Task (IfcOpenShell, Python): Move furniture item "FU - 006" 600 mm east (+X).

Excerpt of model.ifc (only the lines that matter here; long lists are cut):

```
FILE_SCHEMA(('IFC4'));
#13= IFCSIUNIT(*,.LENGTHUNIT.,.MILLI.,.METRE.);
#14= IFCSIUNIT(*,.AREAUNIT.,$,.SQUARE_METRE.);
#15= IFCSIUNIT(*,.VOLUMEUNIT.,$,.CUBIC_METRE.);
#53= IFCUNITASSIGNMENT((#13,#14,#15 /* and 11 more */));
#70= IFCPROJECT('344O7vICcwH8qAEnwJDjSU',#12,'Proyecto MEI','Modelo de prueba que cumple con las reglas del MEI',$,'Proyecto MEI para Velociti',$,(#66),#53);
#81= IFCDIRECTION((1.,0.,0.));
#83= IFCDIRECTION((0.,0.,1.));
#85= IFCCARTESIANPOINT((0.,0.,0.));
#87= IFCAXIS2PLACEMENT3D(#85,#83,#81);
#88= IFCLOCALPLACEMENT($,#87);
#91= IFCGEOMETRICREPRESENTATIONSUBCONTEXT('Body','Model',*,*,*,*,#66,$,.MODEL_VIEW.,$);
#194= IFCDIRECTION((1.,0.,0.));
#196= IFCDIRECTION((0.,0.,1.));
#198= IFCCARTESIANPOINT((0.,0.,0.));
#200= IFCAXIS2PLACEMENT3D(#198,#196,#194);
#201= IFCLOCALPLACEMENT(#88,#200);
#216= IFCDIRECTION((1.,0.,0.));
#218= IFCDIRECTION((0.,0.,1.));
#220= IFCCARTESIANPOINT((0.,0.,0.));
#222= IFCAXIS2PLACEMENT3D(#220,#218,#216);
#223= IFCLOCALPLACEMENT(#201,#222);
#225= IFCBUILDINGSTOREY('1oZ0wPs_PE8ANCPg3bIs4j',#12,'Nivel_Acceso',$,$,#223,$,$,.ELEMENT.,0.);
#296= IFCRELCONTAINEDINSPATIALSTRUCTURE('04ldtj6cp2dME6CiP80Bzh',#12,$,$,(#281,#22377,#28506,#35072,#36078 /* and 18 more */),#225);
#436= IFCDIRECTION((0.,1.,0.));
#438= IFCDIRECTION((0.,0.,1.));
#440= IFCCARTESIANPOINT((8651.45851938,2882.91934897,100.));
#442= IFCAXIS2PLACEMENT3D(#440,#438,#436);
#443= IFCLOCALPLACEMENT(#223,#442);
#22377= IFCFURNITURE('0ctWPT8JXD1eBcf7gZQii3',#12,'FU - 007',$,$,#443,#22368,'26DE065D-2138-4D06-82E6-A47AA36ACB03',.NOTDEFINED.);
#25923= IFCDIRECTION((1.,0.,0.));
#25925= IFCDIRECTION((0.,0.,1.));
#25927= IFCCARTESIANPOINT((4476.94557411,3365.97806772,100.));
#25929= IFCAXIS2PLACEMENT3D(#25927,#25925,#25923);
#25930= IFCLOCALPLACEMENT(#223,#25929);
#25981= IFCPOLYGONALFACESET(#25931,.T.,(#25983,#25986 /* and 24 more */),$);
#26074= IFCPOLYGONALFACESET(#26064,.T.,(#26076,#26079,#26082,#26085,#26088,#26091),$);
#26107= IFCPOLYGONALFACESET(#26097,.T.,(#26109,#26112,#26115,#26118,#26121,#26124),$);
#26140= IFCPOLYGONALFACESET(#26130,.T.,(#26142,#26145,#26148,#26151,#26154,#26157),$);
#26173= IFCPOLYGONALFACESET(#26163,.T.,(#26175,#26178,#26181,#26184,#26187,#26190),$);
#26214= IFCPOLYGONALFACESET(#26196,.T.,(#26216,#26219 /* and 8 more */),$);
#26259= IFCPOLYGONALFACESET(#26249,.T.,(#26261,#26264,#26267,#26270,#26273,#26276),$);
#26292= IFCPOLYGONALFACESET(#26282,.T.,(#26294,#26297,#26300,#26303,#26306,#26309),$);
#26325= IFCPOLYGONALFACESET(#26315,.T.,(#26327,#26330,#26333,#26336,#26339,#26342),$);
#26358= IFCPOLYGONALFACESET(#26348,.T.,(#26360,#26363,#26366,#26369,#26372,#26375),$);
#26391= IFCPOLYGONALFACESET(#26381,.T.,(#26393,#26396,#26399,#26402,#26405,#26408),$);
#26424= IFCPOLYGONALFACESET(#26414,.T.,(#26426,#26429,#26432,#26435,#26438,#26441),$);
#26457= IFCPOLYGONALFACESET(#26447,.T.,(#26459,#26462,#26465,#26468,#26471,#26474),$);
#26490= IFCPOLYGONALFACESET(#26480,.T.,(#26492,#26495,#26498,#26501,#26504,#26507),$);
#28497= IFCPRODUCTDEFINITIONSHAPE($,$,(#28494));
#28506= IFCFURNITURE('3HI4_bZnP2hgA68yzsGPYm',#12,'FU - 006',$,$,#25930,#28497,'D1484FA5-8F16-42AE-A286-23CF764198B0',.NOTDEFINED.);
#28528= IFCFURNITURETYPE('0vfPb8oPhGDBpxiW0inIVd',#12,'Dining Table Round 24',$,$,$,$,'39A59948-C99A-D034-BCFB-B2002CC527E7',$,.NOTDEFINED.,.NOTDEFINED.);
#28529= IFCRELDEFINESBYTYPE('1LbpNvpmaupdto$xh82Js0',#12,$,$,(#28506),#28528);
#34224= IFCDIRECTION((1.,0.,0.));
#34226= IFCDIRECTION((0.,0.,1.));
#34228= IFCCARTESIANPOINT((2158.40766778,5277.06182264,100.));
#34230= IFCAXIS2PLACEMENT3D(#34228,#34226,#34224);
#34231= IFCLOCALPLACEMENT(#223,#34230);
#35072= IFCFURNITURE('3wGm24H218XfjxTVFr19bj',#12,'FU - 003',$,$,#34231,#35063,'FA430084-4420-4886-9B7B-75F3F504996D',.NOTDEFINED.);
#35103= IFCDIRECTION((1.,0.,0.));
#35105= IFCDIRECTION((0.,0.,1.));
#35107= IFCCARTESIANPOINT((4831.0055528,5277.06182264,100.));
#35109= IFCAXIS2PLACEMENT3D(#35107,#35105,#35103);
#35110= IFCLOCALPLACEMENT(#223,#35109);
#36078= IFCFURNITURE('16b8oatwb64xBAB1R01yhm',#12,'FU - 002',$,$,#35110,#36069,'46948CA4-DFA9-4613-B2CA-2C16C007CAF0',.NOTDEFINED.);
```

```python
import ifcopenshell
import ifcopenshell.api.geometry
import ifcopenshell.util.placement
import ifcopenshell.util.unit

model = ifcopenshell.open("model.ifc")
unit_scale = ifcopenshell.util.unit.calculate_unit_scale(model)

item = model.by_guid("3HI4_bZnP2hgA68yzsGPYm")
matrix = ifcopenshell.util.placement.get_local_placement(item.ObjectPlacement)
matrix[0, 3] += 0.6 / unit_scale
ifcopenshell.api.geometry.edit_object_placement(model, product=item, matrix=matrix, is_si=False)

print(ifcopenshell.util.placement.get_local_placement(item.ObjectPlacement).round(3) + 0.0)

model.write("model_v2.ifc")
```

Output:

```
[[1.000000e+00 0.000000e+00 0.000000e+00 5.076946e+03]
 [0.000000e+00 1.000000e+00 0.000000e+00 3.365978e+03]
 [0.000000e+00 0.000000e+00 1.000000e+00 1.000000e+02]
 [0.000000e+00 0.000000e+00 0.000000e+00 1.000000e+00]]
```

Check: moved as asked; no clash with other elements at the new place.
